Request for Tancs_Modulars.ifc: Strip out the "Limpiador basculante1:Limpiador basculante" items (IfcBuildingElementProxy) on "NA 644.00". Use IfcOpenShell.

First a look at what the model holds.

```python
import ifcopenshell
import ifcopenshell.util.element

model = ifcopenshell.open("Tancs_Modulars.ifc")
print(model.schema)
storey = next(s for s in model.by_type("IfcBuildingStorey") if s.Name == "NA 644.00")
proxies = [e for e in ifcopenshell.util.element.get_decomposition(storey) if e.is_a("IfcBuildingElementProxy")]
seen = {}
for e in proxies:
    element_type = ifcopenshell.util.element.get_type(e)
    name = element_type.Name if element_type not in (None, e) else None
    seen[name] = seen.get(name, 0) + 1
for name, count in sorted(seen.items(), key=str):
    print(count, "x", name)
```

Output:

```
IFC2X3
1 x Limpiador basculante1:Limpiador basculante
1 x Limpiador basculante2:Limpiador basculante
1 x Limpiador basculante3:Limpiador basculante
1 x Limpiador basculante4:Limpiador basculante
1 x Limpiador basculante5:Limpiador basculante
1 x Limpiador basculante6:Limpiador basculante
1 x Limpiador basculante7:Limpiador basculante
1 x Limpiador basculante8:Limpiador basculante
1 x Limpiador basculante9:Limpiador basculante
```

```python
import ifcopenshell
import ifcopenshell.api.root
import ifcopenshell.util.element

model = ifcopenshell.open("Tancs_Modulars.ifc")

storey = next(s for s in model.by_type("IfcBuildingStorey") if s.Name == "NA 644.00")
proxies = [e for e in ifcopenshell.util.element.get_decomposition(storey) if e.is_a("IfcBuildingElementProxy")]
targets = [e for e in proxies if (t := ifcopenshell.util.element.get_type(e)) not in (None, e) and t.Name == "Limpiador basculante1:Limpiador basculante"]

for e in targets:
    ifcopenshell.api.root.remove_product(model, product=e)
print(len(targets), "removed")

model.write("Tancs_Modulars_rev.ifc")
```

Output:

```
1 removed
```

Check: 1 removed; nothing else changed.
